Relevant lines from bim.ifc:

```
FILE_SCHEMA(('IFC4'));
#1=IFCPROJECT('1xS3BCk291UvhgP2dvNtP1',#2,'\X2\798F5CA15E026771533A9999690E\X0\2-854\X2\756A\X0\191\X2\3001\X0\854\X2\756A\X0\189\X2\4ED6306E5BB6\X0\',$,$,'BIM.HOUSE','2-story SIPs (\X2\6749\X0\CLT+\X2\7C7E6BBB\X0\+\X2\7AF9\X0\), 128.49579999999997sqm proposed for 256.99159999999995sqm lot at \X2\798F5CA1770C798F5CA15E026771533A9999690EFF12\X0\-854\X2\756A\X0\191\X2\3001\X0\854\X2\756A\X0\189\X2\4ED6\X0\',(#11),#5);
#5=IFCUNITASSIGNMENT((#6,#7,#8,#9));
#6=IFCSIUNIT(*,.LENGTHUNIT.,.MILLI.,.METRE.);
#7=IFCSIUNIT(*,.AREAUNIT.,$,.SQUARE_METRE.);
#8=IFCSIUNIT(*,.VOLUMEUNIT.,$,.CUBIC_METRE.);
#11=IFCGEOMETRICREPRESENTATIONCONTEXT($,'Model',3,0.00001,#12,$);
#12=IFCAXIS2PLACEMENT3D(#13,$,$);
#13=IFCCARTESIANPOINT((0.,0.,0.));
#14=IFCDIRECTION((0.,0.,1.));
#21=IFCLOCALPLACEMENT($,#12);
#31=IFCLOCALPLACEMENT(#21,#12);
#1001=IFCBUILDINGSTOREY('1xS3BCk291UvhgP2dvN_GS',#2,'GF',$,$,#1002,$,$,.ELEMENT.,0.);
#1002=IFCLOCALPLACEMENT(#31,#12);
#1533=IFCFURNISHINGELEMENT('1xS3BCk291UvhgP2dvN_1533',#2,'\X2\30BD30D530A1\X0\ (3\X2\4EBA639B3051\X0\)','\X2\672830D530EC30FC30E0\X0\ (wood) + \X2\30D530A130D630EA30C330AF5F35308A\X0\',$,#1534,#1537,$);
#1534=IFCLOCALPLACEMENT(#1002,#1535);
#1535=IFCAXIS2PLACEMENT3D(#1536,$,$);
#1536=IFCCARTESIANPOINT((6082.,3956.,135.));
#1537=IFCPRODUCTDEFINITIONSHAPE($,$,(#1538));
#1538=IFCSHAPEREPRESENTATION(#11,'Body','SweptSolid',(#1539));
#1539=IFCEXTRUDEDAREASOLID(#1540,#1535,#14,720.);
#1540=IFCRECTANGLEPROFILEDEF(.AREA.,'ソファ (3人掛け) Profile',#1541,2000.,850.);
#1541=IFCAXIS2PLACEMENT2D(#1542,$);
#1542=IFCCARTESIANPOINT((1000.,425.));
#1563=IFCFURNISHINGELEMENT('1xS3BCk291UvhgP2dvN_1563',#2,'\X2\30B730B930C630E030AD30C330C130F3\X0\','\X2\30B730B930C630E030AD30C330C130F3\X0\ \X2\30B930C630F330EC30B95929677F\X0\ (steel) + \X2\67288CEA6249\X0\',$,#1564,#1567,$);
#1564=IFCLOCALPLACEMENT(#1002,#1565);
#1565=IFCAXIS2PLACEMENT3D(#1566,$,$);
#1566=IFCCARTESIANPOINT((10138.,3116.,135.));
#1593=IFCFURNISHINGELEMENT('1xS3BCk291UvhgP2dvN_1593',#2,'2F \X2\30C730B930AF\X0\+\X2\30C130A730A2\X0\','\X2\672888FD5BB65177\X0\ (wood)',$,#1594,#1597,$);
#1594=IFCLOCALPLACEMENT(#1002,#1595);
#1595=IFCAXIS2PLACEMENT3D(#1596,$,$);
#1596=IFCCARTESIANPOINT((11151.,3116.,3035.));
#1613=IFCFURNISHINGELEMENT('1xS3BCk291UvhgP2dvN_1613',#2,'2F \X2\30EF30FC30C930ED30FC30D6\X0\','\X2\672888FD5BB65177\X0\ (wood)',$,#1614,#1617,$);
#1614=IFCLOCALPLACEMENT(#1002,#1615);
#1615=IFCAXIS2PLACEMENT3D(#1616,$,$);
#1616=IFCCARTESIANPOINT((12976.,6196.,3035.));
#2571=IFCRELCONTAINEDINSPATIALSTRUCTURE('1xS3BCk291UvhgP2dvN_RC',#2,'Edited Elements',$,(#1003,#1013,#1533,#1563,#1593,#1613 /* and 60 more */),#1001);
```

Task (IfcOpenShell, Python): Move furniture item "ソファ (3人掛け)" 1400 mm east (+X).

```python
import ifcopenshell
import ifcopenshell.api.geometry
import ifcopenshell.util.placement
import ifcopenshell.util.unit

model = ifcopenshell.open("bim.ifc")
unit_scale = ifcopenshell.util.unit.calculate_unit_scale(model)

item = model.by_guid("1xS3BCk291UvhgP2dvN_1533")
matrix = ifcopenshell.util.placement.get_local_placement(item.ObjectPlacement)
matrix[0, 3] += 1.4 / unit_scale
ifcopenshell.api.geometry.edit_object_placement(model, product=item, matrix=matrix, is_si=False)

print(ifcopenshell.util.placement.get_local_placement(item.ObjectPlacement).round(3) + 0.0)

model.write("bim_updated.ifc")
```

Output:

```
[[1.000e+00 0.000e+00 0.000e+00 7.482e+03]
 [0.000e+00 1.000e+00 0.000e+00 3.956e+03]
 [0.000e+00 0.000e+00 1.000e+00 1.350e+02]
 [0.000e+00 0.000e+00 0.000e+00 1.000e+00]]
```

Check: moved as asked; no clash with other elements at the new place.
